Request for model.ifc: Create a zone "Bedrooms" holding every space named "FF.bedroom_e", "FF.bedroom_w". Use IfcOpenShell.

First a look at what the model holds.

```python
import ifcopenshell

model = ifcopenshell.open("model.ifc")
print(model.schema)
seen = {}
for space in model.by_type("IfcSpace"):
    seen[space.LongName] = seen.get(space.LongName, 0) + 1
for name, count in sorted(seen.items(), key=str):
    print(count, "x", name)
print("zones:", [z.Name for z in model.by_type("IfcZone")][:20])
```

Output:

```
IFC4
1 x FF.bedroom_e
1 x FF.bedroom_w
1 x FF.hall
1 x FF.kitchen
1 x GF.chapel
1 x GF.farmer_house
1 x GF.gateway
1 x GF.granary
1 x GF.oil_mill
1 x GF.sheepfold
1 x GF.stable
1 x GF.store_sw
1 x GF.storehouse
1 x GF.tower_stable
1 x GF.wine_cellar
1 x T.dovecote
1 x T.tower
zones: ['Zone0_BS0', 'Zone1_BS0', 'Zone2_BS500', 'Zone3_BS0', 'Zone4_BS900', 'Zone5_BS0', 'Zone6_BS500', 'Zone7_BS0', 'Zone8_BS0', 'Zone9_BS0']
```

```python
import ifcopenshell
import ifcopenshell.api.group
import ifcopenshell.api.root

model = ifcopenshell.open("model.ifc")

names = {"FF.bedroom_e", "FF.bedroom_w"}
spaces = [s for s in model.by_type("IfcSpace") if s.LongName in names]

zone = ifcopenshell.api.root.create_entity(model, ifc_class="IfcZone", name="Bedrooms")
ifcopenshell.api.group.assign_group(model, products=spaces, group=zone)
print(len(spaces), "spaces in", zone.Name)

model.write("model_edited.ifc")
```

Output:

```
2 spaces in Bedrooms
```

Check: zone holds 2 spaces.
